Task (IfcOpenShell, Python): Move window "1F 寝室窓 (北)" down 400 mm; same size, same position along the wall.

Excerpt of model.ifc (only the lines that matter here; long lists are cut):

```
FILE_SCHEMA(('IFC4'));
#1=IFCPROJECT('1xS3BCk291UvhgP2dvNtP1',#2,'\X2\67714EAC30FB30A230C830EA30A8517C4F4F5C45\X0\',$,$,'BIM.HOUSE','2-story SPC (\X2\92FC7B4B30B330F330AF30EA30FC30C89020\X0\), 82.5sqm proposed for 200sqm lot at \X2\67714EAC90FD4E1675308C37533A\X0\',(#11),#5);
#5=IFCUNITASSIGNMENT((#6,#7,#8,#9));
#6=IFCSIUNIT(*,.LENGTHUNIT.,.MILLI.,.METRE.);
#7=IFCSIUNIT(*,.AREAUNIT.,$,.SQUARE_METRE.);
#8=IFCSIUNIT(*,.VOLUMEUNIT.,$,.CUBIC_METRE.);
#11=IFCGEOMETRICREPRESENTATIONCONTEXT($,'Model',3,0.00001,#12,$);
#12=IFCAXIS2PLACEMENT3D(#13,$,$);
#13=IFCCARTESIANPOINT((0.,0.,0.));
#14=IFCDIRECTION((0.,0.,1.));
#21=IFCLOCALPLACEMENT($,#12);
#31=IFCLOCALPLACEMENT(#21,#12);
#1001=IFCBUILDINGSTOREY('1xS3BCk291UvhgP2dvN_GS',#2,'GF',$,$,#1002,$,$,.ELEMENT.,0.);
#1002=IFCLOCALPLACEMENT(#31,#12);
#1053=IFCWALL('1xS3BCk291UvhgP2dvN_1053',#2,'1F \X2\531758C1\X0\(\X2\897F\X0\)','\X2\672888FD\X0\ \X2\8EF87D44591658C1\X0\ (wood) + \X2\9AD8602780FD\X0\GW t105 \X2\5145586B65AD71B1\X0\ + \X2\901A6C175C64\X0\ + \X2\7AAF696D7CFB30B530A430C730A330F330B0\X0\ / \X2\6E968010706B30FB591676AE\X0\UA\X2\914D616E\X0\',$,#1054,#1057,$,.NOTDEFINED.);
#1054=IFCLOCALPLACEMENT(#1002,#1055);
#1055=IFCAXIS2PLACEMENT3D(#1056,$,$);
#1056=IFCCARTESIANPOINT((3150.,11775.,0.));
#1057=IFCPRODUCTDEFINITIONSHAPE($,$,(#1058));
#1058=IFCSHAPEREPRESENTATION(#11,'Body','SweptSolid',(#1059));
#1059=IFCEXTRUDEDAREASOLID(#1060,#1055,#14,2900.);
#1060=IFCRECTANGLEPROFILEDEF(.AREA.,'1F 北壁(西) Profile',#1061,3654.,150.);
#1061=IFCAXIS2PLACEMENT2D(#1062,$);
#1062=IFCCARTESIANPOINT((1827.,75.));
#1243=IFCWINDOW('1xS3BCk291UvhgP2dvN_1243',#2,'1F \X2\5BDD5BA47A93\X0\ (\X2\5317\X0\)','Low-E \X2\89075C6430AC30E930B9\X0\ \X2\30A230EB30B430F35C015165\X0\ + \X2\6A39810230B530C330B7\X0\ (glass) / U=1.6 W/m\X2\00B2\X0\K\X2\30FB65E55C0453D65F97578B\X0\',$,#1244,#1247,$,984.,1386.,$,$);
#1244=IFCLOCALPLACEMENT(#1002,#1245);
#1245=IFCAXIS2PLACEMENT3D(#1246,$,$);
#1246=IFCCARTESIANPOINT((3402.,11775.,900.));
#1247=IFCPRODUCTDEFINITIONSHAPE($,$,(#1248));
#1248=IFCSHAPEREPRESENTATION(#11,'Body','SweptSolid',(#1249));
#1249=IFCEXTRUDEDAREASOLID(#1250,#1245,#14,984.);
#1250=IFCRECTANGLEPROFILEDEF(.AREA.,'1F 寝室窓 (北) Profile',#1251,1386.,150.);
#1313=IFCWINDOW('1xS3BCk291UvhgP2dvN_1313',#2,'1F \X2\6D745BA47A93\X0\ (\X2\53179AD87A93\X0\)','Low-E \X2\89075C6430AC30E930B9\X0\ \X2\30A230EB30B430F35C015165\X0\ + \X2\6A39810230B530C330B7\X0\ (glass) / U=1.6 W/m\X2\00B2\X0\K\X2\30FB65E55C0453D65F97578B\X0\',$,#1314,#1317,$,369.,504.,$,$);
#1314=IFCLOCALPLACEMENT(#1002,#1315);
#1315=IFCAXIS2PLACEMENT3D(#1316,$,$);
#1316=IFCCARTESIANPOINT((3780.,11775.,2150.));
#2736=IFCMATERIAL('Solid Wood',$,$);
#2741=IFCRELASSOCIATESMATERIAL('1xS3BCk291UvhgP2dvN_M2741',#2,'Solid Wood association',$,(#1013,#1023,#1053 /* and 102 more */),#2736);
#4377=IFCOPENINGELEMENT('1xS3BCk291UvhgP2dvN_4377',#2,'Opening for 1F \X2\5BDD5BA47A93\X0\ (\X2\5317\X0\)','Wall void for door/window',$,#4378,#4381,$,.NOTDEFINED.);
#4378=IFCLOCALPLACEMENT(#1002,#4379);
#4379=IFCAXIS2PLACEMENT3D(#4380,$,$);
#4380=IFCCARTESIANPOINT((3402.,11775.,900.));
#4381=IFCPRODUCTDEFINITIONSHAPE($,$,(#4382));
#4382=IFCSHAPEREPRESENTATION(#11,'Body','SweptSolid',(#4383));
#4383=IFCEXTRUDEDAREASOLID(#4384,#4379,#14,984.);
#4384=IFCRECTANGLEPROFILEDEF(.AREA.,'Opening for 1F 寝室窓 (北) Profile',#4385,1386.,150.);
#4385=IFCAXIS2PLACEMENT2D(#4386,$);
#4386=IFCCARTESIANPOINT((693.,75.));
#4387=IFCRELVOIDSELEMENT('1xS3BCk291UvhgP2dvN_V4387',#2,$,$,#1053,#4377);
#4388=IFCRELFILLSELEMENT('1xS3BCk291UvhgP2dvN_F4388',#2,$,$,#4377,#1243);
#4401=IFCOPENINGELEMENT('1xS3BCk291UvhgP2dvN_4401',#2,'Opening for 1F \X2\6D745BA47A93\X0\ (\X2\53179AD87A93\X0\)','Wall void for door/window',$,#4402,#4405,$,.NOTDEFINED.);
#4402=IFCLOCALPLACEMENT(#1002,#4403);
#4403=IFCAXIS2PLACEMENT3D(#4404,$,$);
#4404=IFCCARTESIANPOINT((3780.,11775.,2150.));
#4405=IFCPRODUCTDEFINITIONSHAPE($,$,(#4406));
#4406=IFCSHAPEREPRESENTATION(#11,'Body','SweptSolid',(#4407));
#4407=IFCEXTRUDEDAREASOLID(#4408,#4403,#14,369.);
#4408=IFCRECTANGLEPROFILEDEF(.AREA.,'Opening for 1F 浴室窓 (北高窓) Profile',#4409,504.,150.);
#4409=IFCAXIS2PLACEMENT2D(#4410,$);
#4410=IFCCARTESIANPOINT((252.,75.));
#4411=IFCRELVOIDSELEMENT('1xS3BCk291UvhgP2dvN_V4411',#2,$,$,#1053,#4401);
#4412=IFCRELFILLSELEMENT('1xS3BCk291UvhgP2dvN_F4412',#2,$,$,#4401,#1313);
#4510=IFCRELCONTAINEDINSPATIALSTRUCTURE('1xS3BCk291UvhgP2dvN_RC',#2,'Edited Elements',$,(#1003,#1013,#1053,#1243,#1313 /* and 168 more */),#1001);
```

```python
import numpy as np
import ifcopenshell
import ifcopenshell.api.geometry
import ifcopenshell.util.placement
import ifcopenshell.util.unit

model = ifcopenshell.open("model.ifc")
unit_scale = ifcopenshell.util.unit.calculate_unit_scale(model)

window = model.by_guid("1xS3BCk291UvhgP2dvN_1243")
opening = window.FillsVoids[0].RelatingOpeningElement
dz = -0.4 / unit_scale

shift = np.array([0.0, 0.0, dz])
# The window is not placed relative to its opening, so move both.
for product in (opening, window):
    matrix = ifcopenshell.util.placement.get_local_placement(product.ObjectPlacement)
    matrix[:3, 3] += shift
    ifcopenshell.api.geometry.edit_object_placement(model, product=product, matrix=matrix, is_si=False)

print(f"moved by {dz * unit_scale:+.3f} m")

model.write("model_v2.ifc")
```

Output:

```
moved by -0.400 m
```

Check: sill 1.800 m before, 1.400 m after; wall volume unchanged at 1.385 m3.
